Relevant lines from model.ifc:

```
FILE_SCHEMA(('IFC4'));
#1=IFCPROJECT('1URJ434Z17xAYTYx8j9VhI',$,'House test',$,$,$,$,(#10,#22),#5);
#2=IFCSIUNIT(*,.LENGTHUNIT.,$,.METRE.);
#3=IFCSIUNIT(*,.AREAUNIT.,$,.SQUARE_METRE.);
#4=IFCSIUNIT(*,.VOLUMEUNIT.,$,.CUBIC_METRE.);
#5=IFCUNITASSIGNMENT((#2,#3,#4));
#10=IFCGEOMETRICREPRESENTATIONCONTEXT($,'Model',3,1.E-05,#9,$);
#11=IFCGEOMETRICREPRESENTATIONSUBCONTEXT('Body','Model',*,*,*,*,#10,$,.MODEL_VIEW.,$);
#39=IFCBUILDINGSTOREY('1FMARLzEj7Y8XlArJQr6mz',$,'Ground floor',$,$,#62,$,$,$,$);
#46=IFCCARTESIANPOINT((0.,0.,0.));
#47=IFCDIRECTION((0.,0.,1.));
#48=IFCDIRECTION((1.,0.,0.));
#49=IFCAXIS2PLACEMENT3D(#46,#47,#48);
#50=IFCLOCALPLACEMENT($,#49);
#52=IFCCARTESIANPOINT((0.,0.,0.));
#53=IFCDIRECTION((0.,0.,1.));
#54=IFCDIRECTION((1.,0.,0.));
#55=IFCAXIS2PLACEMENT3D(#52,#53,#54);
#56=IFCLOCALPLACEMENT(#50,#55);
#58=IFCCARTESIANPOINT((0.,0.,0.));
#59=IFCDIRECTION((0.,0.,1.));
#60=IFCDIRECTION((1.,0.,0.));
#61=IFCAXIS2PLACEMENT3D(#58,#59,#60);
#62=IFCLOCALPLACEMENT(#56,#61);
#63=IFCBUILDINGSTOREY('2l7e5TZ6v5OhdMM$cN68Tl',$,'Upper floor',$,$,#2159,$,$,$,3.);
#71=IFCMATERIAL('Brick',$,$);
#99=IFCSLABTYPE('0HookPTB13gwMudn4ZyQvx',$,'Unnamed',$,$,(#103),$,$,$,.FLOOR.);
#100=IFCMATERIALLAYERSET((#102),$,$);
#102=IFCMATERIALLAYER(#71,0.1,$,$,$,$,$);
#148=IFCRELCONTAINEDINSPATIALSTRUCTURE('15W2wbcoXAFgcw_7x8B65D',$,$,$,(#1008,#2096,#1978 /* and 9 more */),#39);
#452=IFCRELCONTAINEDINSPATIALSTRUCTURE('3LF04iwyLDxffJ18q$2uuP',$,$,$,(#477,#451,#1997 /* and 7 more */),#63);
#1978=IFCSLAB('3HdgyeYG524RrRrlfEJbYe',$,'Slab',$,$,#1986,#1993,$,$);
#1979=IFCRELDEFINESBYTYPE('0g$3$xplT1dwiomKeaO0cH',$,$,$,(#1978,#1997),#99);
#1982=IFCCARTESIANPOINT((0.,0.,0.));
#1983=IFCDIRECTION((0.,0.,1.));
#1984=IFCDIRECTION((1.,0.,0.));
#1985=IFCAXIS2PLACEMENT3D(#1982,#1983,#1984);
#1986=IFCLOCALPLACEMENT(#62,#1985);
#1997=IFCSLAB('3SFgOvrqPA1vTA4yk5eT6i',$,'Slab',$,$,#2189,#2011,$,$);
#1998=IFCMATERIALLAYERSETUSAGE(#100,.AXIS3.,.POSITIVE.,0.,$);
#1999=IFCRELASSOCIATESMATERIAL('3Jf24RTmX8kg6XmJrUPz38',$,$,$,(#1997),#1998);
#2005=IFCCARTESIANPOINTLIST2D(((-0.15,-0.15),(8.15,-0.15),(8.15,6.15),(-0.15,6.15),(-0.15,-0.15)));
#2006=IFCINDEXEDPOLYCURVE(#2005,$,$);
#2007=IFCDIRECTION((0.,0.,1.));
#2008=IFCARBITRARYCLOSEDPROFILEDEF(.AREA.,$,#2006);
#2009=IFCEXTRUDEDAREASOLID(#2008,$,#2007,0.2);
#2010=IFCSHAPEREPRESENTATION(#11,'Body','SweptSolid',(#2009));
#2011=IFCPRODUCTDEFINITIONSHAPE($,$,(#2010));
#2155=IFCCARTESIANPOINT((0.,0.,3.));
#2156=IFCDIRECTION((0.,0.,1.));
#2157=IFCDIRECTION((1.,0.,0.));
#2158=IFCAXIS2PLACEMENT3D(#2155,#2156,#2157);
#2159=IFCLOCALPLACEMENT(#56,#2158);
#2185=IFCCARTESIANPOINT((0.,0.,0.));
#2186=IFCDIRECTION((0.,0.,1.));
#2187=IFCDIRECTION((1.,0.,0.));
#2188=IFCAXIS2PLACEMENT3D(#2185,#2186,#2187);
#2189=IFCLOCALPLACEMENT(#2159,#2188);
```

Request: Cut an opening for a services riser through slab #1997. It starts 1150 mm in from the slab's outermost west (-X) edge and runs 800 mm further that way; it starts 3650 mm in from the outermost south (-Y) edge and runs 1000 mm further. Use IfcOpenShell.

```python
import numpy as np
import ifcopenshell
import ifcopenshell.api.feature
import ifcopenshell.api.geometry
import ifcopenshell.api.root
import ifcopenshell.geom
import ifcopenshell.util.placement
import ifcopenshell.util.representation
import ifcopenshell.util.shape
import ifcopenshell.util.unit

model = ifcopenshell.open("model.ifc")
unit_scale = ifcopenshell.util.unit.calculate_unit_scale(model)
settings = ifcopenshell.geom.settings()


def volume(element):
    """Net volume in cubic metres, openings subtracted."""
    shape = ifcopenshell.geom.create_shape(settings, element)
    return ifcopenshell.util.shape.get_volume(shape.geometry)


slab = model.by_guid("3SFgOvrqPA1vTA4yk5eT6i")
before = volume(slab)

# Extent in the slab's own axes, in metres. The edges named are its -X and -Y sides.
slab_shape = ifcopenshell.geom.create_shape(settings, slab)
vertices = ifcopenshell.util.shape.get_vertices(slab_shape.geometry)
x_min, y_min, bottom = vertices.min(axis=0)
top = vertices[:, 2].max()

opening = ifcopenshell.api.root.create_entity(model, ifc_class="IfcOpeningElement", name="Services riser opening", predefined_type="OPENING")
context = ifcopenshell.util.representation.get_context(model, "Model", "Body", "MODEL_VIEW")
width, depth = 0.8, 1
outline = [(0.0, 0.0), (width, 0.0), (width, depth), (0.0, depth), (0.0, 0.0)]
# Overshoot both faces by 50 mm so the cut is clean.
shape = ifcopenshell.api.geometry.add_slab_representation(
    model, context=context, depth=top - bottom + 0.1, polyline=outline
)
ifcopenshell.api.geometry.assign_representation(model, product=opening, representation=shape)

matrix = ifcopenshell.util.placement.get_local_placement(slab.ObjectPlacement)
matrix[:, 3] = matrix @ np.append(np.array([x_min + 1.15, y_min + 3.65, bottom - 0.05]) / unit_scale, 1.0)
ifcopenshell.api.geometry.edit_object_placement(model, product=opening, matrix=matrix, is_si=False)
ifcopenshell.api.feature.add_feature(model, feature=opening, element=slab)

after = volume(slab)

print(f"slab volume {before:.3f} -> {after:.3f} m3")

model.write("model-out.ifc")
```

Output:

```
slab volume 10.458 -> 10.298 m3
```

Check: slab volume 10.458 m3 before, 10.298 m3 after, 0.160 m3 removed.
